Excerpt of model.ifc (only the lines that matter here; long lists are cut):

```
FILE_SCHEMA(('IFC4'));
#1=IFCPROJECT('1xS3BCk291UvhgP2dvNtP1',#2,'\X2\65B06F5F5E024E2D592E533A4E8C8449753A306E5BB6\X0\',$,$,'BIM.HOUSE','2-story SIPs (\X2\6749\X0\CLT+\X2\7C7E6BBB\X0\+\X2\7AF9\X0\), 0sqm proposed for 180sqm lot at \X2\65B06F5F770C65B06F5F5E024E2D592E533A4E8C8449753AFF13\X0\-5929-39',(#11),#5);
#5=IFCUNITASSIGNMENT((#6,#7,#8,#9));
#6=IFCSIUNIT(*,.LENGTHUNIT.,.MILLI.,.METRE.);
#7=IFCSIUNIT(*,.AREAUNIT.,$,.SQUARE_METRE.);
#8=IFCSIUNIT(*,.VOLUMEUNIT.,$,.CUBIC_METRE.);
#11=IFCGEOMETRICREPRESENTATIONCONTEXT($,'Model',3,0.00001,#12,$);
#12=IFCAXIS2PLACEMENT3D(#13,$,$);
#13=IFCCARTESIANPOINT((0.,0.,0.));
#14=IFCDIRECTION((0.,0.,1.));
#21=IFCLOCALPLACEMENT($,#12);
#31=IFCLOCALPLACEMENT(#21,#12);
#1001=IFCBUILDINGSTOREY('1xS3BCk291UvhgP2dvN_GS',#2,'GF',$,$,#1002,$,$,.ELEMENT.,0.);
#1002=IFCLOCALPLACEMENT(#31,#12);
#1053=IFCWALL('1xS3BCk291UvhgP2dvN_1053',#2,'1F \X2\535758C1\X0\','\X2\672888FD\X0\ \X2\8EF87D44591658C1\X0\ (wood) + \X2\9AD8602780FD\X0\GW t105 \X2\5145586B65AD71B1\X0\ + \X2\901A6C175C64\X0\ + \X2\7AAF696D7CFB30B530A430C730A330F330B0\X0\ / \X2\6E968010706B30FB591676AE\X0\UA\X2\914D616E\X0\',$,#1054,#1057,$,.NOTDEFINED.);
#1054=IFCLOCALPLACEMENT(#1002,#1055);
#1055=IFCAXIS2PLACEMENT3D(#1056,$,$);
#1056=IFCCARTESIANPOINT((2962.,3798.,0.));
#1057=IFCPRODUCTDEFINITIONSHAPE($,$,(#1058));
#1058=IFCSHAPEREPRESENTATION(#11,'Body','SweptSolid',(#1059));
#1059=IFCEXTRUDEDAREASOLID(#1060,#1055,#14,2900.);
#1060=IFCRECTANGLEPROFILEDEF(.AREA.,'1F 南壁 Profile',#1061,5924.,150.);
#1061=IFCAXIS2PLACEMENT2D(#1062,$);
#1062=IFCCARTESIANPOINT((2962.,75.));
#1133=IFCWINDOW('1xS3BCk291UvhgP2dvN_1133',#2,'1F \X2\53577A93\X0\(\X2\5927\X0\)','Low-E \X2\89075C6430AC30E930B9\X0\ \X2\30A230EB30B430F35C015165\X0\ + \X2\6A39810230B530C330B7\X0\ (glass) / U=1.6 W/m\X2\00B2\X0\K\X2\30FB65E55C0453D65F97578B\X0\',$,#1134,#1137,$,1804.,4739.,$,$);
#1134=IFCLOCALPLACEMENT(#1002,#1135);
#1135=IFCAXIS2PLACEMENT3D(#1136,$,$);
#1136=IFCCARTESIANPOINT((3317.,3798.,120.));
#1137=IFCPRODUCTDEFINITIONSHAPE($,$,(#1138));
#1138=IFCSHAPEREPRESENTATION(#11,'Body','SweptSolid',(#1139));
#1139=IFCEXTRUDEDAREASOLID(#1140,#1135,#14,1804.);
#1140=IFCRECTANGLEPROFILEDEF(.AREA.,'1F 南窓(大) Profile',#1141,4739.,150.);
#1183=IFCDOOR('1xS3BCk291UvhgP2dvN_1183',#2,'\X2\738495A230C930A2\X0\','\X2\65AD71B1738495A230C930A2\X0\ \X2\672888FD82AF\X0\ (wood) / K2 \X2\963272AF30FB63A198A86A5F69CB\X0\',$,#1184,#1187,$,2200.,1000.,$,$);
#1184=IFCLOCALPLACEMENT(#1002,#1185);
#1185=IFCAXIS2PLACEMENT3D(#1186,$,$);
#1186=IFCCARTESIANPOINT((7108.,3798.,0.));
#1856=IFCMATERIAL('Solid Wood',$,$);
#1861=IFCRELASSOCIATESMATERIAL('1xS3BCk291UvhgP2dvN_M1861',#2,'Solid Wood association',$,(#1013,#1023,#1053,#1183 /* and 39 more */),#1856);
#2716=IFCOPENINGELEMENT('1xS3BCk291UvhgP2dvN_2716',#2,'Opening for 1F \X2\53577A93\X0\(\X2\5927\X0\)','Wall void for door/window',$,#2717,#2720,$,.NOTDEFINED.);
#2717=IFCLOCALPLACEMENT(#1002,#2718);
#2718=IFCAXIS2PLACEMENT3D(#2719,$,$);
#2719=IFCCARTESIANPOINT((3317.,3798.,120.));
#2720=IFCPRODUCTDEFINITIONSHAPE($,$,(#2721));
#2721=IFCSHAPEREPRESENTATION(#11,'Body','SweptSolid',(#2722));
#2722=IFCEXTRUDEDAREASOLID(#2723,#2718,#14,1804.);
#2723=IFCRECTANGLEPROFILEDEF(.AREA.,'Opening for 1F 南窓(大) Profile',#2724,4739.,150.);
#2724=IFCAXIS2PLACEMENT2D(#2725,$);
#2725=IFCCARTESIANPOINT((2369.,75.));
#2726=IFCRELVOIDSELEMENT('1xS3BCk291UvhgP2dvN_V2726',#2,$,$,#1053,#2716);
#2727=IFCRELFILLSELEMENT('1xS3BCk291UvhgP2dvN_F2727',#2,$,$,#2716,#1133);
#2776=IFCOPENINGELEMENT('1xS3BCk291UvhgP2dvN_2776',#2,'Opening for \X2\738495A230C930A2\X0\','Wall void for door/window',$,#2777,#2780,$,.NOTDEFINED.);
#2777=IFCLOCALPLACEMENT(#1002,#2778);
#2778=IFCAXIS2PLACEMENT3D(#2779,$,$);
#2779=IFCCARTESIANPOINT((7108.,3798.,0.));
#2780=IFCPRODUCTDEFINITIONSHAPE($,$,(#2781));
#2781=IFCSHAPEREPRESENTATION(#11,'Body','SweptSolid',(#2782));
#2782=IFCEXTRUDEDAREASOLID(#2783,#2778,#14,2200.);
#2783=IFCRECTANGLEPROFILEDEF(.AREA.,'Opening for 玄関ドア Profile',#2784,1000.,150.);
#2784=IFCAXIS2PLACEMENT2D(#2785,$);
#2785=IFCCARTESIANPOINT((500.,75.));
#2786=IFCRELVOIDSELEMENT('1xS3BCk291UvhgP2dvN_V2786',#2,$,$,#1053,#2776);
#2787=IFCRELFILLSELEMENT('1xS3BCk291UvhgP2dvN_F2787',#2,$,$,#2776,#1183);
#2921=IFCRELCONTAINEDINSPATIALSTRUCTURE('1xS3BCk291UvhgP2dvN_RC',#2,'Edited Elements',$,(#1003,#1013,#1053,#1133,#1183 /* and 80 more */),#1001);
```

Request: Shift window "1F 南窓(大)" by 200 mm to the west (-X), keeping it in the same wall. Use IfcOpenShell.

```python
import ifcopenshell
import ifcopenshell.api.geometry
import ifcopenshell.util.placement

model = ifcopenshell.open("model.ifc")

window = model.by_id(1133)
opening = window.FillsVoids[0].RelatingOpeningElement
wall = opening.VoidsElements[0].RelatingBuildingElement

wall_matrix = ifcopenshell.util.placement.get_local_placement(wall.ObjectPlacement)
shift = wall_matrix[:3, 0] * -200.0
before = ifcopenshell.util.placement.get_local_placement(window.ObjectPlacement)[:3, 3].copy()

# The window is not placed relative to its opening, so move both.
for product in (opening, window):
    matrix = ifcopenshell.util.placement.get_local_placement(product.ObjectPlacement)
    matrix[:3, 3] += shift
    ifcopenshell.api.geometry.edit_object_placement(model, product=product, matrix=matrix, is_si=False)

after = ifcopenshell.util.placement.get_local_placement(window.ObjectPlacement)[:3, 3]
print("window moved by", (after - before).round(3) + 0.0)

model.write("model_rev.ifc")
```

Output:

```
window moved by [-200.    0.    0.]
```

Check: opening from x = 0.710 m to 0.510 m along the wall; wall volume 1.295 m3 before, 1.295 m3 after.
